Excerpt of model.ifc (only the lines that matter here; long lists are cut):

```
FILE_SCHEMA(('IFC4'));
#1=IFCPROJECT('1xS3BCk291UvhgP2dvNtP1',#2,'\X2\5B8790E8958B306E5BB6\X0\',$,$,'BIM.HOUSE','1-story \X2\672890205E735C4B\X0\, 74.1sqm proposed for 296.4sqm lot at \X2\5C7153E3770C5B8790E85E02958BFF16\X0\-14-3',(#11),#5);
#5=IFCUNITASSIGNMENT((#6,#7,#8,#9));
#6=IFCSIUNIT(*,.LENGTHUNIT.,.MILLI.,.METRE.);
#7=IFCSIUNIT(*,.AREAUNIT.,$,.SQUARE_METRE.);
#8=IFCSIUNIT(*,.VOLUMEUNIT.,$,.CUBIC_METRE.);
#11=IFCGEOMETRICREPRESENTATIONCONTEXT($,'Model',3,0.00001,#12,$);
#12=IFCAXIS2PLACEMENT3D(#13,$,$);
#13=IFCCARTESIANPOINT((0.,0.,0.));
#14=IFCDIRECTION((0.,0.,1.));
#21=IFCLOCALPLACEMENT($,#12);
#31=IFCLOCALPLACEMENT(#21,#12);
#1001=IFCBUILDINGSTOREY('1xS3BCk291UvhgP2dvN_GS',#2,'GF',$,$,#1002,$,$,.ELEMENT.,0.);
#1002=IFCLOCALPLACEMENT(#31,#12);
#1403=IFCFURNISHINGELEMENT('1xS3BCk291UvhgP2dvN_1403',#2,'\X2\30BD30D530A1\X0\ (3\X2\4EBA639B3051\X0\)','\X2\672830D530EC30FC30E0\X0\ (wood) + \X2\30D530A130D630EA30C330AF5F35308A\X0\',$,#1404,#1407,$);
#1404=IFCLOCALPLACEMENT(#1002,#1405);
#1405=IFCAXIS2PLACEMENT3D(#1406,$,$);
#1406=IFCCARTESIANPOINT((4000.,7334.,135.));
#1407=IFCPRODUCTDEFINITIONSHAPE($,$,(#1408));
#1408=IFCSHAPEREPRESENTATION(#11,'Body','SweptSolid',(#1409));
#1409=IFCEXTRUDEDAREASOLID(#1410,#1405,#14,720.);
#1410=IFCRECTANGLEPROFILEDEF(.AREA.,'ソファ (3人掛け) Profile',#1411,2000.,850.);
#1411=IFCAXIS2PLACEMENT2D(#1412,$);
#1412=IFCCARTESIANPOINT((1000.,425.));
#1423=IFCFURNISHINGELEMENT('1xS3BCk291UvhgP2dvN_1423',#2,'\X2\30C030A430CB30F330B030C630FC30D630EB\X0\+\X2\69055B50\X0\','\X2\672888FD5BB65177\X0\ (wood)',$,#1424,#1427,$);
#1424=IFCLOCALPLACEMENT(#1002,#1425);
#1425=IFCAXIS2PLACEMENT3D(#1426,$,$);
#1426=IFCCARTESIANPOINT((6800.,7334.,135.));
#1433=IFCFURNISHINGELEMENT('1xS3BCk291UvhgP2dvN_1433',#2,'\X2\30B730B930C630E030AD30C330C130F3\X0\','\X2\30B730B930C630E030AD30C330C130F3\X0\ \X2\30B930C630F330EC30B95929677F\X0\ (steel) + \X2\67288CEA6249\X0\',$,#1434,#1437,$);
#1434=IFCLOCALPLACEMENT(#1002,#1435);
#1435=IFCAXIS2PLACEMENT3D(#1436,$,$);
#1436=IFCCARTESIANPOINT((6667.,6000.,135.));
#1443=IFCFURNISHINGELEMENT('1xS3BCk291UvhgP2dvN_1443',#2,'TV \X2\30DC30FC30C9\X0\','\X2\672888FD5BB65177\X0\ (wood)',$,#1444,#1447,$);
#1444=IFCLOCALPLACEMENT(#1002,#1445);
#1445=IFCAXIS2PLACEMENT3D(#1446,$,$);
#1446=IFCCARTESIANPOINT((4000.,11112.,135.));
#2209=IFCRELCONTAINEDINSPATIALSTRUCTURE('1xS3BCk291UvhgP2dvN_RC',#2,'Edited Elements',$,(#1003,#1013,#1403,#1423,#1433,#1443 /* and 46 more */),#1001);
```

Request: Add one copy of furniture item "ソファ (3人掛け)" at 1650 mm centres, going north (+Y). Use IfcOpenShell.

```python
import numpy as np
import ifcopenshell
import ifcopenshell.api.geometry
import ifcopenshell.api.root
import ifcopenshell.util.element
import ifcopenshell.util.placement
import ifcopenshell.util.unit

model = ifcopenshell.open("model.ifc")
unit_scale = ifcopenshell.util.unit.calculate_unit_scale(model)


def reuse_history(source, copy):
    """copy_class also copies each property set's owner history, people and application; keep the originals."""
    for rel in copy.IsDefinedBy:
        if rel.is_a("IfcRelDefinesByProperties") and (history := rel.RelatingPropertyDefinition.OwnerHistory):
            rel.RelatingPropertyDefinition.OwnerHistory = source.OwnerHistory
            ifcopenshell.util.element.remove_deep2(model, history)


source = model.by_guid("1xS3BCk291UvhgP2dvN_1403")
base = ifcopenshell.util.placement.get_local_placement(source.ObjectPlacement)
step = np.array([0.0, 1.0, 0.0]) * 1.65 / unit_scale

for i in range(1, 2):
    copy = ifcopenshell.api.root.copy_class(model, product=source)
    copy.Representation = ifcopenshell.util.element.copy_deep(
        model, source.Representation, exclude=["IfcGeometricRepresentationContext", "IfcRepresentationMap"]
    )
    reuse_history(source, copy)
    matrix = base.copy()
    matrix[:3, 3] += i * step
    print("added at", matrix[:3, 3].round(3) + 0.0)
    ifcopenshell.api.geometry.edit_object_placement(model, product=copy, matrix=matrix, is_si=False)

model.write("model_updated.ifc")
```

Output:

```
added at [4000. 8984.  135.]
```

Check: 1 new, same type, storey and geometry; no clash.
